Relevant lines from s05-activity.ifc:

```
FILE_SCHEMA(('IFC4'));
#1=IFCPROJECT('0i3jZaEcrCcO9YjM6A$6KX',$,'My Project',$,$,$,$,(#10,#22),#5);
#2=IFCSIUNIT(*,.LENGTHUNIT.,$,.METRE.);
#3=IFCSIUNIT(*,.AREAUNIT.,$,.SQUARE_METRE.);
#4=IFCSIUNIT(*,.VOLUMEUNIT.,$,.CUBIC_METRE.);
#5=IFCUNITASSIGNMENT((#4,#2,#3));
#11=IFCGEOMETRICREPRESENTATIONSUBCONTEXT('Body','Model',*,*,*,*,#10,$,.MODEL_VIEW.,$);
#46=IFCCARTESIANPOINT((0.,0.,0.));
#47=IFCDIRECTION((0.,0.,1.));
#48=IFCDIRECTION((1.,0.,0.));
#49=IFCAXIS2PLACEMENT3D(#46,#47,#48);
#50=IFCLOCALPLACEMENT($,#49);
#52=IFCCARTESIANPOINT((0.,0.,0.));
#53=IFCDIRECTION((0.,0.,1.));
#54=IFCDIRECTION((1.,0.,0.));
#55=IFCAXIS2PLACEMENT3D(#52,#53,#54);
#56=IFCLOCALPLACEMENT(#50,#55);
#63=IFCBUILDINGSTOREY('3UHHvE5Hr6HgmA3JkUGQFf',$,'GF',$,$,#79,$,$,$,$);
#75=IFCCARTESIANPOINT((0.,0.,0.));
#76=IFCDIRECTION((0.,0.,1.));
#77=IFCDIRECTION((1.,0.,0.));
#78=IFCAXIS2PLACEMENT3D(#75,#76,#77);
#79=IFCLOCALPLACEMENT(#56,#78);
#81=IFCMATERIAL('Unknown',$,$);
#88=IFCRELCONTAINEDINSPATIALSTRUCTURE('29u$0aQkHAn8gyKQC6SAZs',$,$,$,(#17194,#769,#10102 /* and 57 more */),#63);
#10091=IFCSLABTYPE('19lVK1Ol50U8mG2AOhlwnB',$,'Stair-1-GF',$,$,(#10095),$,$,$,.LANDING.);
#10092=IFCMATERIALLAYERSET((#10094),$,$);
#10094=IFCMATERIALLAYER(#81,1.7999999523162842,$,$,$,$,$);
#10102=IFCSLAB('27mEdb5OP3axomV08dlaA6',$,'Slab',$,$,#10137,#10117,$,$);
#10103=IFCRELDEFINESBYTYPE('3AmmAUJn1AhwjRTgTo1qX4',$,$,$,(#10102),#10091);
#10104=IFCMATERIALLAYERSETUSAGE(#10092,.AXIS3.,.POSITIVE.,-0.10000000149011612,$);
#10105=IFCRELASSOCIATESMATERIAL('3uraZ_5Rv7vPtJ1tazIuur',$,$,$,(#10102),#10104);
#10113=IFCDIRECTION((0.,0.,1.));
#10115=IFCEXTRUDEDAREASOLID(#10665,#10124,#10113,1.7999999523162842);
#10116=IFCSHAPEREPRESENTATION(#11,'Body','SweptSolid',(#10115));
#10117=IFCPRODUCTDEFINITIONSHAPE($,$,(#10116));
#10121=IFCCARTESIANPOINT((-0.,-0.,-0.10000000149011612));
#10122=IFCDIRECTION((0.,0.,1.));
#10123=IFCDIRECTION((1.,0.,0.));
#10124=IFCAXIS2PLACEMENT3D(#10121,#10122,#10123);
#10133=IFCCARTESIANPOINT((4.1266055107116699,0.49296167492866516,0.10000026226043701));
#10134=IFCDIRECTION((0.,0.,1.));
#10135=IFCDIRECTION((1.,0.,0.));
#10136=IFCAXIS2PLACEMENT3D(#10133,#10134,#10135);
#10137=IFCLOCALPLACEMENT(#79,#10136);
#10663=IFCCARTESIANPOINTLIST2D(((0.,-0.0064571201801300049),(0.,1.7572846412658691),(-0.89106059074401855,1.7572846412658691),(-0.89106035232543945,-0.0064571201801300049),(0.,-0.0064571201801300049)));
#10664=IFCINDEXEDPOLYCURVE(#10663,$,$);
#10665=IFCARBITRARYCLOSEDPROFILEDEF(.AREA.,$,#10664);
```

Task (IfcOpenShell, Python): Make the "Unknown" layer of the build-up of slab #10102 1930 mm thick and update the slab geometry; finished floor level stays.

```python
import ifcopenshell
import ifcopenshell.util.element
import ifcopenshell.util.representation
import ifcopenshell.util.unit

model = ifcopenshell.open("s05-activity.ifc")
unit_scale = ifcopenshell.util.unit.calculate_unit_scale(model)

layer_set = model.by_id(10092)
layer = next(l for l in layer_set.MaterialLayers if l.Material and l.Material.Name == "Unknown")
change = 1.93 / unit_scale - layer.LayerThickness
layer.LayerThickness += change

# Geometry does not follow the layer set by itself.
slabs = [e for e in ifcopenshell.util.element.get_elements_by_material(model, layer_set) if e.is_a("IfcSlab")]
for slab in sorted(slabs, key=lambda e: e.id()):
    body = ifcopenshell.util.representation.get_representation(slab, "Model", "Body")
    solid = body.Items[0]
    old_depth = solid.Depth
    solid.Depth += change
    # Extruded upwards: lower the start of the extrusion so the top stays.
    x, y, z = solid.Position.Location.Coordinates
    solid.Position.Location = model.createIfcCartesianPoint((x, y, z - change))
    print(slab.id(), f"{old_depth:g} -> {solid.Depth:g}")

# The layers are counted up from the underside, which has moved.
for usage in {ifcopenshell.util.element.get_material(slab) for slab in slabs}:
    usage.OffsetFromReferenceLine -= change

model.write("s05-activity_rev.ifc")
```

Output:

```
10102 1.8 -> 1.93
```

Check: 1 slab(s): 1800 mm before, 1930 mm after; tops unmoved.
